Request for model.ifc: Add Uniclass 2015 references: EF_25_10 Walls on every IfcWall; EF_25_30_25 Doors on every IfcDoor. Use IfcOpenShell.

First a look at what the model holds.

```python
import ifcopenshell

model = ifcopenshell.open("model.ifc")
print(model.schema)
print("classifications:", [c.Name for c in model.by_type("IfcClassification")])
for ifc_class in ("IfcDoor", "IfcRoof", "IfcStair", "IfcWall", "IfcWindow"):
    print(ifc_class, len(model.by_type(ifc_class)))
```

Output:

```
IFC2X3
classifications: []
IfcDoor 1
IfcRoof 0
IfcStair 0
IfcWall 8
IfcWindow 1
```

```python
import ifcopenshell
import ifcopenshell.api.classification

model = ifcopenshell.open("model.ifc")

# IFC2X3 requires Source and Edition and has no link from the project to the system.
system = model.create_entity("IfcClassification", Source="NBS", Edition="2015", Name="Uniclass 2015")

codes = {
    "IfcWall": ("EF_25_10", "Walls"),
    "IfcDoor": ("EF_25_30_25", "Doors"),
}
for ifc_class, (code, name) in codes.items():
    products = model.by_type(ifc_class)
    ifcopenshell.api.classification.add_reference(
        model, products=products, classification=system, identification=code, name=name
    )
    print(code, len(products))

model.write("model_edited.ifc")
```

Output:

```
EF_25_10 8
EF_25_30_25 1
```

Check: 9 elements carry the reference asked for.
